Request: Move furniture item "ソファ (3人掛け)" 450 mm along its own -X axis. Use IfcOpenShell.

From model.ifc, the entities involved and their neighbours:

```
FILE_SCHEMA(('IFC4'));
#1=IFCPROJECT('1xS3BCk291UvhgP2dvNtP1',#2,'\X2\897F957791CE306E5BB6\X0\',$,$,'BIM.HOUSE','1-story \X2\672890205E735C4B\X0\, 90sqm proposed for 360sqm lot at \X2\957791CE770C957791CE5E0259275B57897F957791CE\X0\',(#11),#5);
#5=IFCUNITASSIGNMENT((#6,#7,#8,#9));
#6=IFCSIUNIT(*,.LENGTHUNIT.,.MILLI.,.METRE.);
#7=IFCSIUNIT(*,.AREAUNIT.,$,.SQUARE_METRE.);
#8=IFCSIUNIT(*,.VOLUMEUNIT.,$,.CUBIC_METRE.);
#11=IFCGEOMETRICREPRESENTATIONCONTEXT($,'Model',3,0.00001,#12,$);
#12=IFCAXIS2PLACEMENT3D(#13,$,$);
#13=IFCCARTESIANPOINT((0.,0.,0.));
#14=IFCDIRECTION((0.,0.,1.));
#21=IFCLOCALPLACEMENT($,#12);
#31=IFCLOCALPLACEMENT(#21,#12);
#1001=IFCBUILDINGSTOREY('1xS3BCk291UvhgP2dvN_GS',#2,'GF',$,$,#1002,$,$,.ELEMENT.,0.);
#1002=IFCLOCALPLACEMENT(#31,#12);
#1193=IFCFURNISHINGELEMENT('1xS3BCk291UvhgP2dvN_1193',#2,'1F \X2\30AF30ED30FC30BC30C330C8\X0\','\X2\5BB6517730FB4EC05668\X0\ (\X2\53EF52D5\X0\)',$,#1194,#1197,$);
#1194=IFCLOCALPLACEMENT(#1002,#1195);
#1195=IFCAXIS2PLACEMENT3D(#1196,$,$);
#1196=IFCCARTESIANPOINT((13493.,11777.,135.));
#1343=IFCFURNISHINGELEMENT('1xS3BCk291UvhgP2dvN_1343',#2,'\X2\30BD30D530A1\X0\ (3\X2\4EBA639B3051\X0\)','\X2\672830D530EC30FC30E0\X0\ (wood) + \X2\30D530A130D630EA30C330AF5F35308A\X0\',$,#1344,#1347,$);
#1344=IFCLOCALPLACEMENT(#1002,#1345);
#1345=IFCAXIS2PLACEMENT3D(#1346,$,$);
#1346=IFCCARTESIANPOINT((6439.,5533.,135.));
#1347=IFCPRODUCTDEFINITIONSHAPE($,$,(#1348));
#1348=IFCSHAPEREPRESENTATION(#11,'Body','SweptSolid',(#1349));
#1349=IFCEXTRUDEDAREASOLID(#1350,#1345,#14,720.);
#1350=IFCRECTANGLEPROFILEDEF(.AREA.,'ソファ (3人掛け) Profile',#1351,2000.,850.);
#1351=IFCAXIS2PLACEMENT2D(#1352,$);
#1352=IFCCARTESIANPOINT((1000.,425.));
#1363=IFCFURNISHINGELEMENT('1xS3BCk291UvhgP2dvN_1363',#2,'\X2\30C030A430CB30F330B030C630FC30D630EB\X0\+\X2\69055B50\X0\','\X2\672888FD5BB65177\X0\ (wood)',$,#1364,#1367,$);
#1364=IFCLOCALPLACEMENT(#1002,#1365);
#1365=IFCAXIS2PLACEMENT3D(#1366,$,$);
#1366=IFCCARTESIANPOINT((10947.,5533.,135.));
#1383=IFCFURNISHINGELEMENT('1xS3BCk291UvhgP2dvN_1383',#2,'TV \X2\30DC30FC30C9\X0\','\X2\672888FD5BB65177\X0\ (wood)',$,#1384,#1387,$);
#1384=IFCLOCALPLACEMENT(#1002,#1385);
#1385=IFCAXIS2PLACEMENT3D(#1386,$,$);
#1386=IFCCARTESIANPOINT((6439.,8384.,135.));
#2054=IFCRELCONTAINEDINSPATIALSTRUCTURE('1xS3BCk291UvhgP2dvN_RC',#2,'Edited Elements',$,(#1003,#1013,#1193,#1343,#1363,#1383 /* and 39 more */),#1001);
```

```python
import ifcopenshell
import ifcopenshell.api.geometry
import ifcopenshell.util.placement
import ifcopenshell.util.unit

model = ifcopenshell.open("model.ifc")
unit_scale = ifcopenshell.util.unit.calculate_unit_scale(model)

item = model.by_guid("1xS3BCk291UvhgP2dvN_1343")
matrix = ifcopenshell.util.placement.get_local_placement(item.ObjectPlacement)
matrix[:3, 3] -= matrix[:3, 0] * 0.45 / unit_scale
ifcopenshell.api.geometry.edit_object_placement(model, product=item, matrix=matrix, is_si=False)

print(ifcopenshell.util.placement.get_local_placement(item.ObjectPlacement).round(3) + 0.0)

model.write("model_rev.ifc")
```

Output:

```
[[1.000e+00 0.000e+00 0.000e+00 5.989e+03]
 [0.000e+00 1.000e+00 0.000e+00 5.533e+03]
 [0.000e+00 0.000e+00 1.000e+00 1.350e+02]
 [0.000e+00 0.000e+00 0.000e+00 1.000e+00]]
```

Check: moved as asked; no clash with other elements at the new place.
